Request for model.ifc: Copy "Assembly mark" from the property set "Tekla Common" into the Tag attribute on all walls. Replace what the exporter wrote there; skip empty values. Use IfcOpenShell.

First a look at what the model holds.

```python
import ifcopenshell
import ifcopenshell.util.element

model = ifcopenshell.open("model.ifc")
print(model.schema)
walls = model.by_type("IfcWall")
print(len(walls), "walls")
for e in walls[:8]:
    source = ifcopenshell.util.element.get_pset(e, "Tekla Common", "Assembly mark")
    target = e.Tag
    print(e.id(), repr(source), repr(target), sep=" | ")
```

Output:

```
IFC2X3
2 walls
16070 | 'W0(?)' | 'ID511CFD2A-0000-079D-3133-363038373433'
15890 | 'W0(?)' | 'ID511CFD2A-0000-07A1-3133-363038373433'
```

```python
import ifcopenshell
import ifcopenshell.util.element

model = ifcopenshell.open("model.ifc")

count = 0
for e in model.by_type("IfcWall"):
    value = ifcopenshell.util.element.get_pset(e, "Tekla Common", "Assembly mark")
    current = e.Tag
    if not value or not value.strip() or current == value:
        continue
    e.Tag = value
    count += 1

print(count, "walls updated")

model.write("model_rev.ifc")
```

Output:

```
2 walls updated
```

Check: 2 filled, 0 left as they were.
